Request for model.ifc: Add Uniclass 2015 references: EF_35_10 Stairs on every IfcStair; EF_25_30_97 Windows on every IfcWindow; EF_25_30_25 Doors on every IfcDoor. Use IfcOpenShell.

First a look at what the model holds.

```python
import ifcopenshell

model = ifcopenshell.open("model.ifc")
print(model.schema)
print("classifications:", [c.Name for c in model.by_type("IfcClassification")])
for ifc_class in ("IfcDoor", "IfcRoof", "IfcStair", "IfcWall", "IfcWindow"):
    print(ifc_class, len(model.by_type(ifc_class)))
```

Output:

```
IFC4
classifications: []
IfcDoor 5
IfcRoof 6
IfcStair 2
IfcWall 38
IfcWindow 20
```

```python
import ifcopenshell
import ifcopenshell.api.classification

model = ifcopenshell.open("model.ifc")

system = ifcopenshell.api.classification.add_classification(model, classification="Uniclass 2015")

codes = {
    "IfcStair": ("EF_35_10", "Stairs"),
    "IfcWindow": ("EF_25_30_97", "Windows"),
    "IfcDoor": ("EF_25_30_25", "Doors"),
}
for ifc_class, (code, name) in codes.items():
    products = model.by_type(ifc_class)
    ifcopenshell.api.classification.add_reference(
        model, products=products, classification=system, identification=code, name=name
    )
    print(code, len(products))

model.write("model_v2.ifc")
```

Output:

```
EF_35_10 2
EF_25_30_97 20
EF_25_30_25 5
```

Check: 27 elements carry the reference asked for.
